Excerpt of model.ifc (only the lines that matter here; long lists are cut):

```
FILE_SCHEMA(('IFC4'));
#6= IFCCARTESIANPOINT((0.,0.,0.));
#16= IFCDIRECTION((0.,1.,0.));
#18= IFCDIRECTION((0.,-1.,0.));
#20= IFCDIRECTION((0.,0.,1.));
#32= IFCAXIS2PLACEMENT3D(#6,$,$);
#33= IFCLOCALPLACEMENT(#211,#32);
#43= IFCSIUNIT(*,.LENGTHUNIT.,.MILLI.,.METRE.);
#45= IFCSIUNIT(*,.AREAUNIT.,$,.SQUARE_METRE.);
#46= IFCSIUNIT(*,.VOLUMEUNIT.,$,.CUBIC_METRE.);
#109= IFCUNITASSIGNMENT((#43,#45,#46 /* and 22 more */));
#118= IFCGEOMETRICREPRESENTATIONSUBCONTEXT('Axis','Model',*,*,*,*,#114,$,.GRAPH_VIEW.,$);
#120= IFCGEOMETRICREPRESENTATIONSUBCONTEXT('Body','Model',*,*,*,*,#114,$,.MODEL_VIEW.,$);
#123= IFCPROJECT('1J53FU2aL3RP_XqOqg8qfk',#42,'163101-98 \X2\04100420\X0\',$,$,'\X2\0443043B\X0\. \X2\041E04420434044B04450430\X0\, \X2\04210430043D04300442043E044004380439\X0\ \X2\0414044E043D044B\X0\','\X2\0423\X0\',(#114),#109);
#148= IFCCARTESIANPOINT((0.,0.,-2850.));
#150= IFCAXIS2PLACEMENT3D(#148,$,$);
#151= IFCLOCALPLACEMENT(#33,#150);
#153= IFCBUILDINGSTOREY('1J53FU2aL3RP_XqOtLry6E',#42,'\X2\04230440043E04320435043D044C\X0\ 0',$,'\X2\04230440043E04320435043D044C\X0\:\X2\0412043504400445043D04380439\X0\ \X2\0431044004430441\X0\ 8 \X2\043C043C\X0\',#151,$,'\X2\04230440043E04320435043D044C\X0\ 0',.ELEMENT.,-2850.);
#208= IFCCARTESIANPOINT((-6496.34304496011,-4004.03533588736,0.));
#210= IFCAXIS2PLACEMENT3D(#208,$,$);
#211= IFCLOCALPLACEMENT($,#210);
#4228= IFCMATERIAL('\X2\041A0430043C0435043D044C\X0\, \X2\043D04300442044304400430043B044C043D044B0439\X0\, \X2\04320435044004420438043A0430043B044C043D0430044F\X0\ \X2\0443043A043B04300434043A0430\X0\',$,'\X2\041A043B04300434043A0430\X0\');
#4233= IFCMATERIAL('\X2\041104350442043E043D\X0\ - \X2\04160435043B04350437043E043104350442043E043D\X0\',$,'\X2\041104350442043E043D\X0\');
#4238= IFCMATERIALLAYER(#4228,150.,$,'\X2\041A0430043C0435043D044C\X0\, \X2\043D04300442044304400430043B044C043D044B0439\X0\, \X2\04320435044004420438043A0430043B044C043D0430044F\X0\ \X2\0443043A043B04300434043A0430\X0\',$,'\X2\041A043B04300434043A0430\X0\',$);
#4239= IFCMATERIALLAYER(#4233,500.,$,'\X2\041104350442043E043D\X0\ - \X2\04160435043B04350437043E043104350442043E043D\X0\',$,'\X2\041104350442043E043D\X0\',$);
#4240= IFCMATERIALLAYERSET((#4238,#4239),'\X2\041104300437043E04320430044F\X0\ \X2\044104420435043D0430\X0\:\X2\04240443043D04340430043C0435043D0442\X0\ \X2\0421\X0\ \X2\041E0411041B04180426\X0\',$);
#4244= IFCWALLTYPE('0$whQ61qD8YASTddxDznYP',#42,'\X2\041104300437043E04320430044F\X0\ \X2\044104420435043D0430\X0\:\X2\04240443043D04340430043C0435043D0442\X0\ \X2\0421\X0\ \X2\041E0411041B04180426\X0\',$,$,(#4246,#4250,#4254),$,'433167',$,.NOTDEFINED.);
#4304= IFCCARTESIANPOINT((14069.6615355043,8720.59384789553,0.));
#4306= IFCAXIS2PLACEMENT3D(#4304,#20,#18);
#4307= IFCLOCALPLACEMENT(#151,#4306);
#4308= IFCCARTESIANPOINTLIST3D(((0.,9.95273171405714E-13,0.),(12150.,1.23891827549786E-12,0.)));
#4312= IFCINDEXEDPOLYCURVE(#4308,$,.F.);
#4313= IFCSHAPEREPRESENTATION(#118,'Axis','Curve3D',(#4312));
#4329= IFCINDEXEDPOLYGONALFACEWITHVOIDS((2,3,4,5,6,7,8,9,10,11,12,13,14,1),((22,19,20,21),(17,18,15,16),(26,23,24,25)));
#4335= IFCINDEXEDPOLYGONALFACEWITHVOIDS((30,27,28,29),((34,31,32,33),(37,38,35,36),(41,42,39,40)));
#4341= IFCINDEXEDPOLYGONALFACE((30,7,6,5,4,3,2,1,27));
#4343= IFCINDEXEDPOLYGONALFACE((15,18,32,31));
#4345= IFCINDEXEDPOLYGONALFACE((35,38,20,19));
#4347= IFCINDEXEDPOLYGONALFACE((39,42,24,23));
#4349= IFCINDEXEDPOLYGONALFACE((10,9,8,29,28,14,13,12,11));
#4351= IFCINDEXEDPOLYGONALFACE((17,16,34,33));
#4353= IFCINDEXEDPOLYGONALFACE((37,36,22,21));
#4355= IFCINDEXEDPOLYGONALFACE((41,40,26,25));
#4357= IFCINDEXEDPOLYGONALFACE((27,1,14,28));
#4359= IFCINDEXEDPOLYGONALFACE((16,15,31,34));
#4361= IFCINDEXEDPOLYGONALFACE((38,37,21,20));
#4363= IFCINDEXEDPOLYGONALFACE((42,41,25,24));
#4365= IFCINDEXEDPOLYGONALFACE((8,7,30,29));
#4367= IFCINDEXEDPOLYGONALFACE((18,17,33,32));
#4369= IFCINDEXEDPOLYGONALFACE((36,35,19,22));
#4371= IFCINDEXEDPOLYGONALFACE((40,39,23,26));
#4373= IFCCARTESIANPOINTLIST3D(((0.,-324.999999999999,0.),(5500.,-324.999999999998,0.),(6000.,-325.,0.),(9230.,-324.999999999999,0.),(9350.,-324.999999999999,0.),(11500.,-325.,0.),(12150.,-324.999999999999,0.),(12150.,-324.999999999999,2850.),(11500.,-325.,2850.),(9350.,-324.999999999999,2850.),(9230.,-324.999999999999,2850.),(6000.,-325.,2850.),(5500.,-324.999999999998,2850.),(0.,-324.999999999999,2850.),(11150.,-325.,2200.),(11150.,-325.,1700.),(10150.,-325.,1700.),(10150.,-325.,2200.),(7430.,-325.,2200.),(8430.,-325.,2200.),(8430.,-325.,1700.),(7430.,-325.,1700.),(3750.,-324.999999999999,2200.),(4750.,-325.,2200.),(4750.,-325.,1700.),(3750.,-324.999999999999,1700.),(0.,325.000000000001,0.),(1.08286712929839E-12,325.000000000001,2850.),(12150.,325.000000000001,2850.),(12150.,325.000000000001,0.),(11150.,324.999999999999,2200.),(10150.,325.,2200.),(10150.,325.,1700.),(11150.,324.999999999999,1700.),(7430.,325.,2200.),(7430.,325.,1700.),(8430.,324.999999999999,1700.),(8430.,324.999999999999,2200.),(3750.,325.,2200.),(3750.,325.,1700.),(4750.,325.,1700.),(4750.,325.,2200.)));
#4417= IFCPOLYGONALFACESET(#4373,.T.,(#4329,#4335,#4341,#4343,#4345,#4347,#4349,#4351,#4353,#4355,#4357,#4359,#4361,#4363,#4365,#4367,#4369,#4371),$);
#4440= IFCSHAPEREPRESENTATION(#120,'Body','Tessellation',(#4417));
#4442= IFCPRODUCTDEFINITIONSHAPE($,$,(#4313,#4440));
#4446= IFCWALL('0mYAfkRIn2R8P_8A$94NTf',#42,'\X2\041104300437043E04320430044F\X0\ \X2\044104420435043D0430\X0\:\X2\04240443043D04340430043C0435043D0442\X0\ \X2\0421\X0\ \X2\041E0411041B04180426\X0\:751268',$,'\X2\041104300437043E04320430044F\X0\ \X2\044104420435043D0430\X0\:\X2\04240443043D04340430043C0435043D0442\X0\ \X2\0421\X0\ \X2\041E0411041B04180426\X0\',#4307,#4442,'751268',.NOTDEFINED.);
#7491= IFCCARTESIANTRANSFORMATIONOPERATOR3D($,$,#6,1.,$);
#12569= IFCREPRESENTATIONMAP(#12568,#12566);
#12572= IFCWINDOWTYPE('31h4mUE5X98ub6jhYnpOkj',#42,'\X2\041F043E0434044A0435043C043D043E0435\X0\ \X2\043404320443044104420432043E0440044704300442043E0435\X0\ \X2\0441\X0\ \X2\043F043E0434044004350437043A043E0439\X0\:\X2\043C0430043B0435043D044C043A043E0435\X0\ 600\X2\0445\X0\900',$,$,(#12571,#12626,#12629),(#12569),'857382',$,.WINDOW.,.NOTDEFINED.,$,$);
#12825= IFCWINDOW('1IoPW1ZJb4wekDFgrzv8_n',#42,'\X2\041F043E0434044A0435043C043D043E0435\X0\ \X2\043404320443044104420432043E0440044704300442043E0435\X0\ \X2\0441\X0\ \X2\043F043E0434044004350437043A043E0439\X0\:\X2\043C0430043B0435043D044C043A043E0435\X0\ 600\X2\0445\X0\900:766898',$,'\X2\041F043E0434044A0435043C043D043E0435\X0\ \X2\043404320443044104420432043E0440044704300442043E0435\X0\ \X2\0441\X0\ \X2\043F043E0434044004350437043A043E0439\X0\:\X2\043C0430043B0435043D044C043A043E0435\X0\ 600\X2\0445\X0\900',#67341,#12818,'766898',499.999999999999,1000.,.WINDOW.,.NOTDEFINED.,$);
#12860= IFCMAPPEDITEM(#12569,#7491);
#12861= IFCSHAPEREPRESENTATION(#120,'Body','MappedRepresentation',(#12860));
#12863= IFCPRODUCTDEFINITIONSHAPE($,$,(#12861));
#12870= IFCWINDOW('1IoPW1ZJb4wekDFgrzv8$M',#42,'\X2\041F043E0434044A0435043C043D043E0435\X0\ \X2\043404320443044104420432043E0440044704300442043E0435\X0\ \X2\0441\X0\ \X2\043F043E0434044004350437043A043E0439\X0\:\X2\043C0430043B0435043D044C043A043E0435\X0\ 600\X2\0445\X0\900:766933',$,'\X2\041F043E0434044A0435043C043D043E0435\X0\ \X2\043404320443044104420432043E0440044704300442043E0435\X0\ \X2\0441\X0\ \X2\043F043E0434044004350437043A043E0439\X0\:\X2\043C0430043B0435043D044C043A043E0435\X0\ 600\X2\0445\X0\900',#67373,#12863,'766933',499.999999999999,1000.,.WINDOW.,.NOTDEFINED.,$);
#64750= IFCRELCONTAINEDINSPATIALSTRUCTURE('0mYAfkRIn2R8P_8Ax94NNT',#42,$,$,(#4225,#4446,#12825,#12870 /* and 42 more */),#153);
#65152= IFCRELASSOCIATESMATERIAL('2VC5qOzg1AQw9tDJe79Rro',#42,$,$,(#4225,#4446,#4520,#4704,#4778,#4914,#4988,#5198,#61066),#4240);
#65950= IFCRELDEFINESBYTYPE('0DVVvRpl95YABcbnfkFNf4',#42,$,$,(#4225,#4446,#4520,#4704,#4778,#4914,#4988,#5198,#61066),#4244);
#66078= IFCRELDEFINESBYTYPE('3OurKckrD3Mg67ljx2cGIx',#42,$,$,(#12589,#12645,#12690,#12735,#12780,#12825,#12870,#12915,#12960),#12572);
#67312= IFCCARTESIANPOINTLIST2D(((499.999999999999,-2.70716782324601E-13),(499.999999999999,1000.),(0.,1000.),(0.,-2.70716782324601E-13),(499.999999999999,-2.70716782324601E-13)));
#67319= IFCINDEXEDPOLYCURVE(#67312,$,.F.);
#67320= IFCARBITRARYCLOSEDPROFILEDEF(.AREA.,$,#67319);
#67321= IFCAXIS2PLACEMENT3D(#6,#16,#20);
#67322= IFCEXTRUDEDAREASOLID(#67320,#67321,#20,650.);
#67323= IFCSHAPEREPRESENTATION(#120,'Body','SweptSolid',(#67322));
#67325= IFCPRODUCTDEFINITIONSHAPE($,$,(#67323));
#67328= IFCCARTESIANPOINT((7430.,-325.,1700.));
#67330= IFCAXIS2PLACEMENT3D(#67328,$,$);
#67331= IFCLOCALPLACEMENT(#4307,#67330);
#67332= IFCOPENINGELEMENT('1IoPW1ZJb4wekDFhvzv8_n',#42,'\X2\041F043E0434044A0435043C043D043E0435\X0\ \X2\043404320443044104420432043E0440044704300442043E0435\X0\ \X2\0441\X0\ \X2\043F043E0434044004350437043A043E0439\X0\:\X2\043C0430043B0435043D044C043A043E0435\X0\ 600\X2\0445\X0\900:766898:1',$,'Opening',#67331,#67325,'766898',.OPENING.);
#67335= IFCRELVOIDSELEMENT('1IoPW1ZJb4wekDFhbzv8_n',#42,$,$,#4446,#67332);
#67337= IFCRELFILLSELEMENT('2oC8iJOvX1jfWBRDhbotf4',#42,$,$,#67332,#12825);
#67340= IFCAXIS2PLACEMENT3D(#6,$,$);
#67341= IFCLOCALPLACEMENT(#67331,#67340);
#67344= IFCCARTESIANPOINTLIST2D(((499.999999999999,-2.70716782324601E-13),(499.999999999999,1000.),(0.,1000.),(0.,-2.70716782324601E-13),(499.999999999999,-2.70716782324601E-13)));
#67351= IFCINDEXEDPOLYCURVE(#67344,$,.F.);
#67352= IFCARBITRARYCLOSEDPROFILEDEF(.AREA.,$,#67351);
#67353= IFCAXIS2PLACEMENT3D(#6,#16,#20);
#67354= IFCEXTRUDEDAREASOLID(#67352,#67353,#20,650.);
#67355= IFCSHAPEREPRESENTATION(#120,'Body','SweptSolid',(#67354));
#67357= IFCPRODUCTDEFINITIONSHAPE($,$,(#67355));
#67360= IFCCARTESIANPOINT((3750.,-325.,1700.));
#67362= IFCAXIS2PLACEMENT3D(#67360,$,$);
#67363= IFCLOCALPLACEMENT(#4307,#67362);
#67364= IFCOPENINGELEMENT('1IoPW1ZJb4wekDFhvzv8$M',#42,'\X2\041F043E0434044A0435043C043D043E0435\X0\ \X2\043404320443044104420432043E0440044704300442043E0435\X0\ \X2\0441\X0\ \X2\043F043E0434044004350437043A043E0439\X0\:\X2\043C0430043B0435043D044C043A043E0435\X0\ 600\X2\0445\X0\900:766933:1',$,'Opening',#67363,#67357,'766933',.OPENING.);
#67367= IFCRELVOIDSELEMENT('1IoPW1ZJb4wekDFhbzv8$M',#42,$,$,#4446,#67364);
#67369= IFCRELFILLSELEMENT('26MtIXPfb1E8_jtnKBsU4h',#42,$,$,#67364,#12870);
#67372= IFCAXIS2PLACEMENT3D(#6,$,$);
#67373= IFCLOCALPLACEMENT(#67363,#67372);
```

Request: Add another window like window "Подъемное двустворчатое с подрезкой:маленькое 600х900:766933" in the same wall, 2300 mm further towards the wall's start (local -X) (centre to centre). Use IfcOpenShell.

```python
import ifcopenshell
import ifcopenshell.api.feature
import ifcopenshell.api.geometry
import ifcopenshell.api.root
import ifcopenshell.geom
import ifcopenshell.util.element
import ifcopenshell.util.placement
import ifcopenshell.util.shape

model = ifcopenshell.open("model.ifc")
settings = ifcopenshell.geom.settings()


def volume(element):
    """Net volume in cubic metres, openings subtracted."""
    shape = ifcopenshell.geom.create_shape(settings, element)
    return ifcopenshell.util.shape.get_volume(shape.geometry)


def reuse_history(source, copy):
    """copy_class also copies each property set's owner history, people and application; keep the originals."""
    for rel in copy.IsDefinedBy:
        if rel.is_a("IfcRelDefinesByProperties") and (history := rel.RelatingPropertyDefinition.OwnerHistory):
            rel.RelatingPropertyDefinition.OwnerHistory = source.OwnerHistory
            ifcopenshell.util.element.remove_deep2(model, history)


window = model.by_id(12870)
opening = window.FillsVoids[0].RelatingOpeningElement
wall = opening.VoidsElements[0].RelatingBuildingElement
before = volume(wall)
shift = ifcopenshell.util.placement.get_local_placement(wall.ObjectPlacement)[:3, 0] * -2300.0

# copy_class copies the void relationship, type, container and properties, but no geometry.
new_opening = ifcopenshell.api.root.copy_class(model, product=opening)
new_opening.Representation = ifcopenshell.util.element.copy_deep(
    model, opening.Representation, exclude=["IfcGeometricRepresentationContext", "IfcRepresentationMap"]
)
new_opening.Name = "Подъемное двустворчатое с подрезкой:маленькое 600х900"
new_opening.Tag = None
new_window = ifcopenshell.api.root.copy_class(model, product=window)
new_window.Representation = ifcopenshell.util.element.copy_deep(
    model, window.Representation, exclude=["IfcGeometricRepresentationContext", "IfcRepresentationMap"]
)
new_window.Name = "Подъемное двустворчатое с подрезкой:маленькое 600х900"
new_window.Tag = None
reuse_history(window, new_window)
ifcopenshell.api.feature.add_filling(model, opening=new_opening, element=new_window)

for old, new in ((opening, new_opening), (window, new_window)):
    matrix = ifcopenshell.util.placement.get_local_placement(old.ObjectPlacement)
    matrix[:3, 3] += shift
    ifcopenshell.api.geometry.edit_object_placement(model, product=new, matrix=matrix, is_si=False)

after = volume(wall)

print(f"wall volume {before:.3f} -> {after:.3f} m3")

model.write("model_edited.ifc")
```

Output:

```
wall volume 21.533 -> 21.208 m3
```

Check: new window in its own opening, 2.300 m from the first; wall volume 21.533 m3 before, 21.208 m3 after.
